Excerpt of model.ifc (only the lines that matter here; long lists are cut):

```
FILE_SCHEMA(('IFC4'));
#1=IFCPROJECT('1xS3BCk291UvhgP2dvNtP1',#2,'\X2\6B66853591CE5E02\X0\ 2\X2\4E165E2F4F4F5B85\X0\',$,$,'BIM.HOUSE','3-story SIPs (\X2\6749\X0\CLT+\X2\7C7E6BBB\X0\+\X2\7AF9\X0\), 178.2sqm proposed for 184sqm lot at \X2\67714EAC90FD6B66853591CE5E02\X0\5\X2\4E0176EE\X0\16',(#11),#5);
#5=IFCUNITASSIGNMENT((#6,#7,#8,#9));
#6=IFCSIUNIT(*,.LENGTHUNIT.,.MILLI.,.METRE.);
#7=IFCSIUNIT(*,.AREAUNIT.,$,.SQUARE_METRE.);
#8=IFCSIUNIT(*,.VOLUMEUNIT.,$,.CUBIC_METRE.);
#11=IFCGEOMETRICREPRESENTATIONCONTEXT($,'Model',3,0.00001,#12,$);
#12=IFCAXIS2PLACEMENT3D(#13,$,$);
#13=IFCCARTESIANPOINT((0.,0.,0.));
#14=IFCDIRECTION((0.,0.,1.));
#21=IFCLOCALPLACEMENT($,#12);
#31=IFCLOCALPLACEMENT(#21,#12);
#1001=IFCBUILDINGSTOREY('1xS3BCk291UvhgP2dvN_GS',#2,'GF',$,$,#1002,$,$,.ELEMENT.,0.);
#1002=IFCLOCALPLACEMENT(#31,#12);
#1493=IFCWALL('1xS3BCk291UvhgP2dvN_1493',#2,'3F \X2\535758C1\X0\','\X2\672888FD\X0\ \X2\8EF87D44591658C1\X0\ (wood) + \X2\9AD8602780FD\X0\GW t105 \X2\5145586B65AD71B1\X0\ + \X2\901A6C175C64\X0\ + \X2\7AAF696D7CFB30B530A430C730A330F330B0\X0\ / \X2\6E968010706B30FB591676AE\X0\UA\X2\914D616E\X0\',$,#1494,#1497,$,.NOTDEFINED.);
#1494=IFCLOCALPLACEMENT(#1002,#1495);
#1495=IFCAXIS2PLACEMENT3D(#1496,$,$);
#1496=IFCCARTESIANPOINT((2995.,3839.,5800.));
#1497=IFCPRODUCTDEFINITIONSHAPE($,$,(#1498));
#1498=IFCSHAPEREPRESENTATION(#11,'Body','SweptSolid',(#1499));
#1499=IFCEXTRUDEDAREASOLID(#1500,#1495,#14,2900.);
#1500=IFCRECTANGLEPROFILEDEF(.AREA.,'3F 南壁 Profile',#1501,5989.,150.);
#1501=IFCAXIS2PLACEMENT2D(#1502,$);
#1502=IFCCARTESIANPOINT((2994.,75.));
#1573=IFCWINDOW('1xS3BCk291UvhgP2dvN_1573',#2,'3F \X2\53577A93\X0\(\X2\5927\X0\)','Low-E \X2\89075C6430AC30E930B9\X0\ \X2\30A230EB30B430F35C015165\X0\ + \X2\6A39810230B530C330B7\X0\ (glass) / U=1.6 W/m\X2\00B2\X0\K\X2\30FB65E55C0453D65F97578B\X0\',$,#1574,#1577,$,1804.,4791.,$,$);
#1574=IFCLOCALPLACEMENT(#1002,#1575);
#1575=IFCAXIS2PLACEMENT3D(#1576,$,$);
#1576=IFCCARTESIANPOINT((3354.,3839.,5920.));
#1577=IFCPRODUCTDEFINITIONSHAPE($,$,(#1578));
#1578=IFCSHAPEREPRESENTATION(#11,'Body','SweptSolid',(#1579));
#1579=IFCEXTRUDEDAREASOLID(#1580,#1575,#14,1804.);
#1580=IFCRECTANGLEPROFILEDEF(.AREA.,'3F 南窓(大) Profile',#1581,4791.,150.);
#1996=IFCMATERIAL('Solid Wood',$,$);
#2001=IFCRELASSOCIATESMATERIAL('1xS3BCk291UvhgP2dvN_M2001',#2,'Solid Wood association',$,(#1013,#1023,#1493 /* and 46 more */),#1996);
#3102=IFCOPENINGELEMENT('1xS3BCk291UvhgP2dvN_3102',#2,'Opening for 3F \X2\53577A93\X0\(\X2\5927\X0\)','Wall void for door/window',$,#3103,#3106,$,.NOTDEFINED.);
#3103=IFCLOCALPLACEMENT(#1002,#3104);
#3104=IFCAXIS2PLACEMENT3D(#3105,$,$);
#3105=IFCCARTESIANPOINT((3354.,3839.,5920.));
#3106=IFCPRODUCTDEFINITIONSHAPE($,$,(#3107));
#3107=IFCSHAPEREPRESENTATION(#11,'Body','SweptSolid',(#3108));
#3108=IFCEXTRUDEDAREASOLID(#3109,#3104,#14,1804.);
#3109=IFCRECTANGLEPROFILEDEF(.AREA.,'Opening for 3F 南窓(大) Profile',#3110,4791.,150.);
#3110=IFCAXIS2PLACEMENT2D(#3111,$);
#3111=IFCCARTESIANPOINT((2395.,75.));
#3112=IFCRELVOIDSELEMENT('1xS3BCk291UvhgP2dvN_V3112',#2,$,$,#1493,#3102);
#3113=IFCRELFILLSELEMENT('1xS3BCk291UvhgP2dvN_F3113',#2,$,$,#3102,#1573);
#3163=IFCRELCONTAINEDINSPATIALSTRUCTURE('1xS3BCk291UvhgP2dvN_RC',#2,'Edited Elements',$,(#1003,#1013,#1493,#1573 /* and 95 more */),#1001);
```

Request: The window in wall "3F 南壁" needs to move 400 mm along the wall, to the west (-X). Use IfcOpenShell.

```python
import ifcopenshell
import ifcopenshell.api.geometry
import ifcopenshell.util.placement
import ifcopenshell.util.unit

model = ifcopenshell.open("model.ifc")
unit_scale = ifcopenshell.util.unit.calculate_unit_scale(model)

window = model.by_id(1573)
opening = window.FillsVoids[0].RelatingOpeningElement
wall = opening.VoidsElements[0].RelatingBuildingElement

wall_matrix = ifcopenshell.util.placement.get_local_placement(wall.ObjectPlacement)
shift = wall_matrix[:3, 0] * -0.4 / unit_scale
before = ifcopenshell.util.placement.get_local_placement(window.ObjectPlacement)[:3, 3].copy()

# The window is not placed relative to its opening, so move both.
for product in (opening, window):
    matrix = ifcopenshell.util.placement.get_local_placement(product.ObjectPlacement)
    matrix[:3, 3] += shift
    ifcopenshell.api.geometry.edit_object_placement(model, product=product, matrix=matrix, is_si=False)

after = ifcopenshell.util.placement.get_local_placement(window.ObjectPlacement)[:3, 3]
print("window moved by", (after - before).round(3) + 0.0)

model.write("model_updated.ifc")
```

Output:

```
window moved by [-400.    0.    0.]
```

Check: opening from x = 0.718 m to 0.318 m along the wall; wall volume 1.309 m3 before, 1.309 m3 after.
